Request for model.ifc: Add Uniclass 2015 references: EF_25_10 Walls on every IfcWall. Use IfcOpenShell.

First a look at what the model holds.

```python
import ifcopenshell

model = ifcopenshell.open("model.ifc")
print(model.schema)
print("classifications:", [c.Name for c in model.by_type("IfcClassification")])
for ifc_class in ("IfcDoor", "IfcRoof", "IfcStair", "IfcWall", "IfcWindow"):
    print(ifc_class, len(model.by_type(ifc_class)))
```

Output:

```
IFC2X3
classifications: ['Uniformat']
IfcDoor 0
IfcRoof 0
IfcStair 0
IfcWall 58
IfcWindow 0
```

```python
import ifcopenshell
import ifcopenshell.api.classification

model = ifcopenshell.open("model.ifc")

# IFC2X3 requires Source and Edition and has no link from the project to the system.
system = model.create_entity("IfcClassification", Source="NBS", Edition="2015", Name="Uniclass 2015")

codes = {
    "IfcWall": ("EF_25_10", "Walls"),
}
for ifc_class, (code, name) in codes.items():
    products = model.by_type(ifc_class)
    ifcopenshell.api.classification.add_reference(
        model, products=products, classification=system, identification=code, name=name
    )
    print(code, len(products))

model.write("model_updated.ifc")
```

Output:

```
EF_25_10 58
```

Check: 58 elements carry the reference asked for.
